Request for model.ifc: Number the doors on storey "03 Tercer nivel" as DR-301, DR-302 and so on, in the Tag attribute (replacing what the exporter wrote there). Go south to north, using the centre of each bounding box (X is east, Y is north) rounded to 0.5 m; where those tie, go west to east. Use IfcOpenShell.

First a look at what the model holds.

```python
import ifcopenshell
import ifcopenshell.util.element
import ifcopenshell.util.placement

model = ifcopenshell.open("model.ifc")
print(model.schema)
storey = next(s for s in model.by_type("IfcBuildingStorey") if s.Name == "03 Tercer nivel")
doors = [e for e in ifcopenshell.util.element.get_decomposition(storey) if e.is_a("IfcDoor")]
for e in sorted(doors, key=lambda e: e.id()):
    origin = ifcopenshell.util.placement.get_local_placement(e.ObjectPlacement)[:3, 3]
    print(e.id(), e.Tag, e.Name, origin.round(2) + 0.0, sep=" | ")
```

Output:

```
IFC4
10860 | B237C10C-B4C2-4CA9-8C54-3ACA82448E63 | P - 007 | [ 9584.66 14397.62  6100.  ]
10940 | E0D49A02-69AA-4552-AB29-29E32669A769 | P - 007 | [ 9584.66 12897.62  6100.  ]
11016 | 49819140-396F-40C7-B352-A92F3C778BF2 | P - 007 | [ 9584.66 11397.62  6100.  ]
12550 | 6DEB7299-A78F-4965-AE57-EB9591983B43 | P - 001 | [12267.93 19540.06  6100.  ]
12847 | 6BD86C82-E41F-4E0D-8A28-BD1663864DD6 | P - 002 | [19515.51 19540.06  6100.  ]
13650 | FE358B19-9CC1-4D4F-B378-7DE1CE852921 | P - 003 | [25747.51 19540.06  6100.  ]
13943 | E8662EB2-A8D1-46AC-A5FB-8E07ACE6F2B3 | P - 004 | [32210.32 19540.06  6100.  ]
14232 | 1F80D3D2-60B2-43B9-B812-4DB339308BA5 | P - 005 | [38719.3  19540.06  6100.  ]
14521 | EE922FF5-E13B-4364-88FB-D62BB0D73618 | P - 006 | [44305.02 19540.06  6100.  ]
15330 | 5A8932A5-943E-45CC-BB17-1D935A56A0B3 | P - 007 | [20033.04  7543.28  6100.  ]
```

```python
import ifcopenshell
import ifcopenshell.geom
import ifcopenshell.util.element
import ifcopenshell.util.shape

model = ifcopenshell.open("model.ifc")
settings = ifcopenshell.geom.settings()
settings.set("use-world-coords", True)


def centre(element):
    shape = ifcopenshell.geom.create_shape(settings, element)
    return ifcopenshell.util.shape.get_bbox_centroid(shape.geometry)


storey = next(s for s in model.by_type("IfcBuildingStorey") if s.Name == "03 Tercer nivel")
doors = [e for e in ifcopenshell.util.element.get_decomposition(storey) if e.is_a("IfcDoor")]

# Insertion points can sit at a corner or the storey origin, so sort by the geometry (in metres).
centres = {e: centre(e) for e in doors}
doors.sort(key=lambda e: (round(centres[e][1] / 0.5), centres[e][0]))

for i, e in enumerate(doors, start=1):
    number = f"DR-3{i:02d}"
    e.Tag = number
    print(e.id(), number)

model.write("model-out.ifc")
```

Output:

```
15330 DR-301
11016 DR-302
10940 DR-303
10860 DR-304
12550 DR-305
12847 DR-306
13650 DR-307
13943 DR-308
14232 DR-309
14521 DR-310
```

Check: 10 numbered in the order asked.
